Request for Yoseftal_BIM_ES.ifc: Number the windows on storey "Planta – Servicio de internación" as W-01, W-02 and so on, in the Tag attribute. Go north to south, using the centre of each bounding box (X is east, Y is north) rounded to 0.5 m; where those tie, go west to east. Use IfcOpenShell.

First a look at what the model holds.

```python
import ifcopenshell
import ifcopenshell.util.element
import ifcopenshell.util.placement

model = ifcopenshell.open("Yoseftal_BIM_ES.ifc")
print(model.schema)
storey = next(s for s in model.by_type("IfcBuildingStorey") if s.Name == "Planta – Servicio de internación")
windows = [e for e in ifcopenshell.util.element.get_decomposition(storey) if e.is_a("IfcWindow")]
for e in sorted(windows, key=lambda e: e.id()):
    origin = ifcopenshell.util.placement.get_local_placement(e.ObjectPlacement)[:3, 3]
    print(e.id(), e.Tag, e.Name, origin.round(2) + 0.0, sep=" | ")
```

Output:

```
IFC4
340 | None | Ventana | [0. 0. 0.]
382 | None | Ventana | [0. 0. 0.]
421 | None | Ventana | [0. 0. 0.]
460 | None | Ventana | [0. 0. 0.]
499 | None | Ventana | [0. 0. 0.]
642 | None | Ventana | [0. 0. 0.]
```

```python
import ifcopenshell
import ifcopenshell.geom
import ifcopenshell.util.element
import ifcopenshell.util.shape

model = ifcopenshell.open("Yoseftal_BIM_ES.ifc")
settings = ifcopenshell.geom.settings()
settings.set("use-world-coords", True)


def centre(element):
    shape = ifcopenshell.geom.create_shape(settings, element)
    return ifcopenshell.util.shape.get_bbox_centroid(shape.geometry)


storey = next(s for s in model.by_type("IfcBuildingStorey") if s.Name == "Planta – Servicio de internación")
windows = [e for e in ifcopenshell.util.element.get_decomposition(storey) if e.is_a("IfcWindow")]

# Insertion points can sit at a corner or the storey origin, so sort by the geometry (in metres).
centres = {e: centre(e) for e in windows}
windows.sort(key=lambda e: (-round(centres[e][1] / 0.5), centres[e][0]))

for i, e in enumerate(windows, start=1):
    number = f"W-{i:02d}"
    e.Tag = number
    print(e.id(), number)

model.write("Yoseftal_BIM_ES-out.ifc")
```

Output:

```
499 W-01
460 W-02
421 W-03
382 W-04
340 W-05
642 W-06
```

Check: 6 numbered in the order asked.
